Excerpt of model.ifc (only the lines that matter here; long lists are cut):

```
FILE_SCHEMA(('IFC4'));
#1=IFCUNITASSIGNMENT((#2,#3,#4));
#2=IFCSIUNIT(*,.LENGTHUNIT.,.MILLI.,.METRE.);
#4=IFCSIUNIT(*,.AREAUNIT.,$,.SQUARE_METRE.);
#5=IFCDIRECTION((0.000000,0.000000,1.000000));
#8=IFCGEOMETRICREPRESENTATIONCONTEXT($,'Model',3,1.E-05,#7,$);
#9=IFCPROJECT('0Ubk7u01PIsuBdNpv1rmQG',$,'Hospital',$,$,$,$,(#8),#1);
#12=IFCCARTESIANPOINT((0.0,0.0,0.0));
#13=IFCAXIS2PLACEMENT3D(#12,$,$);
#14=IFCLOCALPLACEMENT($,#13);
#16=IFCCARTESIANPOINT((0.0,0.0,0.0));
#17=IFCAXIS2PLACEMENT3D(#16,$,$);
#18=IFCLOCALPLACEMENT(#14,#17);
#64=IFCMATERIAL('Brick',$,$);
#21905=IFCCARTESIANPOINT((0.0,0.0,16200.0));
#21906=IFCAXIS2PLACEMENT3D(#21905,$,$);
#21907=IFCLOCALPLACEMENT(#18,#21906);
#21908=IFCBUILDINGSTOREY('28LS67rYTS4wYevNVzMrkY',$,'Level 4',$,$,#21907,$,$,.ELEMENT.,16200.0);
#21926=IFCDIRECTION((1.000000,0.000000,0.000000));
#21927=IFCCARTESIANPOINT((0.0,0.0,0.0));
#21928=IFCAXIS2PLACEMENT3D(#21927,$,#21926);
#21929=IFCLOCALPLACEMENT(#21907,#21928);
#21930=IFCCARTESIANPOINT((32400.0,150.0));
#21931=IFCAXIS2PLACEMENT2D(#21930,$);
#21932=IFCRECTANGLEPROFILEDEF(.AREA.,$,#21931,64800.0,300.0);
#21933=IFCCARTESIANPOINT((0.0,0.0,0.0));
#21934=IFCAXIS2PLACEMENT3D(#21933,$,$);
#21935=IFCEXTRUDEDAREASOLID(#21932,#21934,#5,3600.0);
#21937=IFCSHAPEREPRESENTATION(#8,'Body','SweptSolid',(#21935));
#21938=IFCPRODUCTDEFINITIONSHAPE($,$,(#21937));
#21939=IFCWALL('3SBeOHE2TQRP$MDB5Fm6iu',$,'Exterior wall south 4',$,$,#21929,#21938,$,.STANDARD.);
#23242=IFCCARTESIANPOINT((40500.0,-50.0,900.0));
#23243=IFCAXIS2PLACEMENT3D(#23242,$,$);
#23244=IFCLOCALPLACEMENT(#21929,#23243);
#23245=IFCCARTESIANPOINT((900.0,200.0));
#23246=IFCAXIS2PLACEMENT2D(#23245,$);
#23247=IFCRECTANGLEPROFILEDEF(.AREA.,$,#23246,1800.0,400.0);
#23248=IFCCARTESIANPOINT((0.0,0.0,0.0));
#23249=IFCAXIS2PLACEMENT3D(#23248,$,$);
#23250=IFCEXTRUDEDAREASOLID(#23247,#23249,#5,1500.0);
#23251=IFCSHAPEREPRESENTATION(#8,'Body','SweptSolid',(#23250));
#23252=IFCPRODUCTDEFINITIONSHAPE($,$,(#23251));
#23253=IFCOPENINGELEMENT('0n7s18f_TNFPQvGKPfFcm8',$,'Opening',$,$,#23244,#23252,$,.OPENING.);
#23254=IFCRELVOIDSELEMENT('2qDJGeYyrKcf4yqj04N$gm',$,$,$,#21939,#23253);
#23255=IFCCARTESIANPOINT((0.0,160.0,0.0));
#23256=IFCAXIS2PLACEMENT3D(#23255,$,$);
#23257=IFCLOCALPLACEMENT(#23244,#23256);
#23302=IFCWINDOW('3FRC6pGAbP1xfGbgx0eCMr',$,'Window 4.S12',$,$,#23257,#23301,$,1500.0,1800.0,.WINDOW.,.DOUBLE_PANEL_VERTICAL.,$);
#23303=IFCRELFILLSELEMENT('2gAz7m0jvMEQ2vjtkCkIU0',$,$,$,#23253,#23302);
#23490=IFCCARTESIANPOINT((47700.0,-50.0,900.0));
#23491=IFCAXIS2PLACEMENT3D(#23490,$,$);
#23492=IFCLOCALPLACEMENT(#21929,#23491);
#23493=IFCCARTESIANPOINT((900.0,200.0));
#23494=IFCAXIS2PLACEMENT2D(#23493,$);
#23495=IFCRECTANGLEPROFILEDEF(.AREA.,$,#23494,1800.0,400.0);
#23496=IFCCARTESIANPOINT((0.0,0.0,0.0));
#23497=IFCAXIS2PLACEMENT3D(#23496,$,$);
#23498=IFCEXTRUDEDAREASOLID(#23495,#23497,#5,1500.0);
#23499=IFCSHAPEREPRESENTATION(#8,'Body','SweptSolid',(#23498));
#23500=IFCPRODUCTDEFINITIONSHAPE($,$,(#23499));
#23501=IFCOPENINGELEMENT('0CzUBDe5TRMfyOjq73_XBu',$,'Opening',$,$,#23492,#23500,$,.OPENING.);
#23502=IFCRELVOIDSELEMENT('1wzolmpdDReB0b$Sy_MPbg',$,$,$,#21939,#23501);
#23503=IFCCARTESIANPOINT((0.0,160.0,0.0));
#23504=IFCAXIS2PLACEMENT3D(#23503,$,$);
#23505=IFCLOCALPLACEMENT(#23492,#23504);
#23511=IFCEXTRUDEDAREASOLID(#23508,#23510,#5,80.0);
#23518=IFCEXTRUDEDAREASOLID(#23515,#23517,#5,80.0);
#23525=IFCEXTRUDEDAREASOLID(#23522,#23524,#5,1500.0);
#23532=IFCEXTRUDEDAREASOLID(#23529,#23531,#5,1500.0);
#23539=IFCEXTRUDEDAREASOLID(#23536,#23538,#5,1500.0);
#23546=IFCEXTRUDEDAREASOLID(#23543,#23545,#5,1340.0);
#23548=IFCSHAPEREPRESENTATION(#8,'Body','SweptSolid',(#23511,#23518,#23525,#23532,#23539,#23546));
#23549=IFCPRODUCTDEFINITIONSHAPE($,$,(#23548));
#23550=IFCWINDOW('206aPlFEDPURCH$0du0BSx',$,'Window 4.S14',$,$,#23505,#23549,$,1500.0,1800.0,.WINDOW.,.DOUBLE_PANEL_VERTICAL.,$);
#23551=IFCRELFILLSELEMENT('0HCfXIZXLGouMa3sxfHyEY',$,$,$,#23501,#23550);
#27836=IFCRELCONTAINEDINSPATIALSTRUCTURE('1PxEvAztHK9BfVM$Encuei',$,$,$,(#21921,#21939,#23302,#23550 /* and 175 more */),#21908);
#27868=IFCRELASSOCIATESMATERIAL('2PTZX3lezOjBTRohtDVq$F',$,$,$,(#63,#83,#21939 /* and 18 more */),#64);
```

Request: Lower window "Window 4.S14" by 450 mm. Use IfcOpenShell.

```python
import numpy as np
import ifcopenshell
import ifcopenshell.api.geometry
import ifcopenshell.util.placement
import ifcopenshell.util.unit

model = ifcopenshell.open("model.ifc")
unit_scale = ifcopenshell.util.unit.calculate_unit_scale(model)

window = model.by_guid("206aPlFEDPURCH$0du0BSx")
opening = window.FillsVoids[0].RelatingOpeningElement
dz = -0.45 / unit_scale

shift = np.array([0.0, 0.0, dz])
# The window is placed relative to its opening, so it follows when the opening moves.
matrix = ifcopenshell.util.placement.get_local_placement(opening.ObjectPlacement)
matrix[:3, 3] += shift
ifcopenshell.api.geometry.edit_object_placement(
    model, product=opening, matrix=matrix, is_si=False, should_transform_children=True
)

print(f"moved by {dz * unit_scale:+.3f} m")

model.write("model_updated.ifc")
```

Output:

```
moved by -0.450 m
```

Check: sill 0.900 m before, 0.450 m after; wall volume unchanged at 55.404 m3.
